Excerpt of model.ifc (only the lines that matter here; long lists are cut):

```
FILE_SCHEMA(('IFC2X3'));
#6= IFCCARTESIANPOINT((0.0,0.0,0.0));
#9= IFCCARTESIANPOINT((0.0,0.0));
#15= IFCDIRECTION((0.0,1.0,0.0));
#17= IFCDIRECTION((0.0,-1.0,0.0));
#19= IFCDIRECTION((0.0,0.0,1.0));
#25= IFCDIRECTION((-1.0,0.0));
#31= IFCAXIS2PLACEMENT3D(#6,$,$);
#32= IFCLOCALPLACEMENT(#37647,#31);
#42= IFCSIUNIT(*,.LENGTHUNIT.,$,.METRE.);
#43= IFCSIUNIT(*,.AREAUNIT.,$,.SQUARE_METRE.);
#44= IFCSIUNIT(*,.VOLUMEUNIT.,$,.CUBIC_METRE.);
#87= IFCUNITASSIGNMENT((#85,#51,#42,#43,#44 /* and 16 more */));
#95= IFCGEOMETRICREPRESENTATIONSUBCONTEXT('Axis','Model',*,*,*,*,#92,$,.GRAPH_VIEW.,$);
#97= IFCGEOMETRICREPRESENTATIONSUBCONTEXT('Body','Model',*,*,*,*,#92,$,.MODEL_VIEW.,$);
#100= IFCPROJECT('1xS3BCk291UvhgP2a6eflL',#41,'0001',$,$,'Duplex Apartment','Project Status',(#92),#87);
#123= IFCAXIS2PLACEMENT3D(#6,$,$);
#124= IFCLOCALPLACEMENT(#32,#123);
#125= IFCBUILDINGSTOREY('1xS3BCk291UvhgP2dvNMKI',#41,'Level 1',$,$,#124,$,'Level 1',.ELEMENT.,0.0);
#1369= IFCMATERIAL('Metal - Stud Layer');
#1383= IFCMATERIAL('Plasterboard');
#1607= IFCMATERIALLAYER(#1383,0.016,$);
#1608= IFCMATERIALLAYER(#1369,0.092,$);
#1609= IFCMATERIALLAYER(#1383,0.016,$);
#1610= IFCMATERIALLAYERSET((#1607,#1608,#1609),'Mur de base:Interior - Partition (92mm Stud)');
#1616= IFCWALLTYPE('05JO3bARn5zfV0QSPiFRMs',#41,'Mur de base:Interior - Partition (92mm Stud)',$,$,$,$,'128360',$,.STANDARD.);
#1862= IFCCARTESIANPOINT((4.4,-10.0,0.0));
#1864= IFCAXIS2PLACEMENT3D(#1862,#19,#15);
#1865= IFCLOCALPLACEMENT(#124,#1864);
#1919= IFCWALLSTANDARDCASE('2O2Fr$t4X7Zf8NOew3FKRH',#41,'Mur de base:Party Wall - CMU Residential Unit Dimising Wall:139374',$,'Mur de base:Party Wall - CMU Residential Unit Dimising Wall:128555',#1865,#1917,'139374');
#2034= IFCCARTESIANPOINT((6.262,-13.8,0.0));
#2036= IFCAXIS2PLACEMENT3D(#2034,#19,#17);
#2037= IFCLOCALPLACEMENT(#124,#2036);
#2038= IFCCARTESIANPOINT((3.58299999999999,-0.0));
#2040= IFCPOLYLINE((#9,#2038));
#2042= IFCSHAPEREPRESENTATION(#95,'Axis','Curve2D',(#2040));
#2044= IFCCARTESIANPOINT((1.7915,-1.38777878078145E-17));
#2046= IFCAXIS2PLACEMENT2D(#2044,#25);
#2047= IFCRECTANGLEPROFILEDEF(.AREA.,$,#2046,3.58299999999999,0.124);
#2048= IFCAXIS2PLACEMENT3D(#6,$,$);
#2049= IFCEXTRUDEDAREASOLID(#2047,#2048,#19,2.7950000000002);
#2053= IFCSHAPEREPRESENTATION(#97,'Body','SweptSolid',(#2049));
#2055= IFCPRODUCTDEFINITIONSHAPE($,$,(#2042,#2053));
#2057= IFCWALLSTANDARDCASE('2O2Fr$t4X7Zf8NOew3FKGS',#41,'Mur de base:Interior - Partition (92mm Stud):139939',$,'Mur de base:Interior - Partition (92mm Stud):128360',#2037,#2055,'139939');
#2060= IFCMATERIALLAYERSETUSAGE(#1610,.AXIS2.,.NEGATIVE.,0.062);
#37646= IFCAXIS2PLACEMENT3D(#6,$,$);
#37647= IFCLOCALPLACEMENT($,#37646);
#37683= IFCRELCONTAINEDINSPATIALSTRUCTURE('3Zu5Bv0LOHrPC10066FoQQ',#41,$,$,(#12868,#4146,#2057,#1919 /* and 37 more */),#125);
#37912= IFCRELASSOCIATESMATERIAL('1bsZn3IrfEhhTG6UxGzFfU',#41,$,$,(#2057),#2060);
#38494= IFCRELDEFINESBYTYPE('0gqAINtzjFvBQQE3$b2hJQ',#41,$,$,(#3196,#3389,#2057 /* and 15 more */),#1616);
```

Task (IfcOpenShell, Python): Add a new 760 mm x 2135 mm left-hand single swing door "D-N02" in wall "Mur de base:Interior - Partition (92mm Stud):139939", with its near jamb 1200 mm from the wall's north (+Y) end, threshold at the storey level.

```python
import numpy as np
import ifcopenshell
import ifcopenshell.api.feature
import ifcopenshell.api.geometry
import ifcopenshell.api.root
import ifcopenshell.api.spatial
import ifcopenshell.api.type
import ifcopenshell.geom
import ifcopenshell.util.element
import ifcopenshell.util.placement
import ifcopenshell.util.representation
import ifcopenshell.util.shape
import ifcopenshell.util.unit

model = ifcopenshell.open("model.ifc")
unit_scale = ifcopenshell.util.unit.calculate_unit_scale(model)
settings = ifcopenshell.geom.settings()


def volume(element):
    """Net volume in cubic metres, openings subtracted."""
    shape = ifcopenshell.geom.create_shape(settings, element)
    return ifcopenshell.util.shape.get_volume(shape.geometry)


wall = model.by_guid("2O2Fr$t4X7Zf8NOew3FKGS")
storey = ifcopenshell.util.element.get_container(wall, ifc_class="IfcBuildingStorey")
context = ifcopenshell.util.representation.get_context(model, "Model", "Body", "MODEL_VIEW")
before = volume(wall)

width, height, from_end, sill = 0.76, 2.135, 1.2, 0.0  # metres

# The wall runs along its own X axis, and the end named is its -X end.
wall_shape = ifcopenshell.geom.create_shape(settings, wall)
x, y, z = ifcopenshell.util.shape.get_vertices(wall_shape.geometry).T
start = x.min() + from_end
face, thickness = float(y.min()), float(y.max() - y.min())
wall_matrix = ifcopenshell.util.placement.get_local_placement(wall.ObjectPlacement)
level = ifcopenshell.util.placement.get_local_placement(storey.ObjectPlacement)[2, 3]


def in_wall(x, y):
    """Placement at x, y metres in the wall's axes, at sill height."""
    matrix = wall_matrix.copy()
    matrix[:, 3] = wall_matrix @ np.array([x / unit_scale, y / unit_scale, 0.0, 1.0])
    matrix[2, 3] = level + sill / unit_scale
    return matrix


# Opening: a box that overshoots both wall faces by 50 mm.
opening = ifcopenshell.api.root.create_entity(model, ifc_class="IfcOpeningElement")
box = ifcopenshell.api.geometry.add_wall_representation(
    model, context=context, length=width, height=height, thickness=thickness + 0.1
)
ifcopenshell.api.geometry.assign_representation(model, product=opening, representation=box)
ifcopenshell.api.geometry.edit_object_placement(model, product=opening, matrix=in_wall(start, face - 0.05), is_si=False)
ifcopenshell.api.feature.add_feature(model, feature=opening, element=wall)

door = ifcopenshell.api.root.create_entity(model, ifc_class="IfcDoor", name="D-N02")
door.OverallWidth, door.OverallHeight = width / unit_scale, height / unit_scale
body = ifcopenshell.api.geometry.add_door_representation(
    model,
    context=context,
    overall_width=door.OverallWidth,
    overall_height=door.OverallHeight,
    operation_type="SINGLE_SWING_LEFT",
    lining_properties={"LiningDepth": thickness / unit_scale, "ThresholdDepth": thickness / unit_scale},
)
ifcopenshell.api.geometry.assign_representation(model, product=door, representation=body)
ifcopenshell.api.spatial.assign_container(model, products=[door], relating_structure=storey)
fills = ifcopenshell.api.feature.add_filling(model, opening=opening, element=door)
fills.OwnerHistory = door.OwnerHistory  # required in IFC2X3

# IFC2X3 keeps the operation on the door style.
style = ifcopenshell.api.root.create_entity(model, ifc_class="IfcDoorStyle", name="D-N02")
style.OperationType, style.ConstructionType = "SINGLE_SWING_LEFT", "NOTDEFINED"
style.ParameterTakesPrecedence = style.Sizeable = False
ifcopenshell.api.type.assign_type(model, related_objects=[door], relating_type=style)

# The lining spans the wall, so the door starts at the wall face.
ifcopenshell.api.geometry.edit_object_placement(model, product=door, matrix=in_wall(start, face), is_si=False)

after = volume(wall)

print(f"wall volume {before:.3f} -> {after:.3f} m3")

model.write("model_v2.ifc")
```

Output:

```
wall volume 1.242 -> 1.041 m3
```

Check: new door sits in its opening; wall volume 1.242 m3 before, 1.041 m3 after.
